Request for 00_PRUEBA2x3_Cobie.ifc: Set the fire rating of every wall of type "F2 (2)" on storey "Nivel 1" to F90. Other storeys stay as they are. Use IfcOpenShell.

First a look at what the model holds.

```python
import ifcopenshell
import ifcopenshell.util.element

model = ifcopenshell.open("00_PRUEBA2x3_Cobie.ifc")
print(model.schema)
storey = next(s for s in model.by_type("IfcBuildingStorey") if s.Name == "Nivel 1")
walls = [e for e in ifcopenshell.util.element.get_decomposition(storey) if e.is_a("IfcWall")]
seen = {}
for e in walls:
    element_type = ifcopenshell.util.element.get_type(e)
    key = (element_type.Name if element_type != e and element_type else None, ifcopenshell.util.element.get_pset(e, "Pset_WallCommon", "FireRating"))
    seen[key] = seen.get(key, 0) + 1
for (name, value), count in sorted(seen.items(), key=str):
    print(count, "x", name, "|", value)
```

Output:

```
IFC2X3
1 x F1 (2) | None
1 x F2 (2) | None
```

```python
import ifcopenshell
import ifcopenshell.api.pset
import ifcopenshell.util.element

model = ifcopenshell.open("00_PRUEBA2x3_Cobie.ifc")

storey = next(s for s in model.by_type("IfcBuildingStorey") if s.Name == "Nivel 1")
walls = [e for e in ifcopenshell.util.element.get_decomposition(storey) if e.is_a("IfcWall")]

count = 0
for e in walls:
    element_type = ifcopenshell.util.element.get_type(e)
    if element_type in (None, e) or element_type.Name != "F2 (2)":
        continue
    # add_pset returns the element's existing set when there is one.
    pset = ifcopenshell.api.pset.add_pset(model, product=e, name="Pset_WallCommon")
    ifcopenshell.api.pset.edit_pset(model, pset=pset, properties={"FireRating": "F90"})
    count += 1

print(count, "walls updated")

model.write("00_PRUEBA2x3_Cobie_v2.ifc")
```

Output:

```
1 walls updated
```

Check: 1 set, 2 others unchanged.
